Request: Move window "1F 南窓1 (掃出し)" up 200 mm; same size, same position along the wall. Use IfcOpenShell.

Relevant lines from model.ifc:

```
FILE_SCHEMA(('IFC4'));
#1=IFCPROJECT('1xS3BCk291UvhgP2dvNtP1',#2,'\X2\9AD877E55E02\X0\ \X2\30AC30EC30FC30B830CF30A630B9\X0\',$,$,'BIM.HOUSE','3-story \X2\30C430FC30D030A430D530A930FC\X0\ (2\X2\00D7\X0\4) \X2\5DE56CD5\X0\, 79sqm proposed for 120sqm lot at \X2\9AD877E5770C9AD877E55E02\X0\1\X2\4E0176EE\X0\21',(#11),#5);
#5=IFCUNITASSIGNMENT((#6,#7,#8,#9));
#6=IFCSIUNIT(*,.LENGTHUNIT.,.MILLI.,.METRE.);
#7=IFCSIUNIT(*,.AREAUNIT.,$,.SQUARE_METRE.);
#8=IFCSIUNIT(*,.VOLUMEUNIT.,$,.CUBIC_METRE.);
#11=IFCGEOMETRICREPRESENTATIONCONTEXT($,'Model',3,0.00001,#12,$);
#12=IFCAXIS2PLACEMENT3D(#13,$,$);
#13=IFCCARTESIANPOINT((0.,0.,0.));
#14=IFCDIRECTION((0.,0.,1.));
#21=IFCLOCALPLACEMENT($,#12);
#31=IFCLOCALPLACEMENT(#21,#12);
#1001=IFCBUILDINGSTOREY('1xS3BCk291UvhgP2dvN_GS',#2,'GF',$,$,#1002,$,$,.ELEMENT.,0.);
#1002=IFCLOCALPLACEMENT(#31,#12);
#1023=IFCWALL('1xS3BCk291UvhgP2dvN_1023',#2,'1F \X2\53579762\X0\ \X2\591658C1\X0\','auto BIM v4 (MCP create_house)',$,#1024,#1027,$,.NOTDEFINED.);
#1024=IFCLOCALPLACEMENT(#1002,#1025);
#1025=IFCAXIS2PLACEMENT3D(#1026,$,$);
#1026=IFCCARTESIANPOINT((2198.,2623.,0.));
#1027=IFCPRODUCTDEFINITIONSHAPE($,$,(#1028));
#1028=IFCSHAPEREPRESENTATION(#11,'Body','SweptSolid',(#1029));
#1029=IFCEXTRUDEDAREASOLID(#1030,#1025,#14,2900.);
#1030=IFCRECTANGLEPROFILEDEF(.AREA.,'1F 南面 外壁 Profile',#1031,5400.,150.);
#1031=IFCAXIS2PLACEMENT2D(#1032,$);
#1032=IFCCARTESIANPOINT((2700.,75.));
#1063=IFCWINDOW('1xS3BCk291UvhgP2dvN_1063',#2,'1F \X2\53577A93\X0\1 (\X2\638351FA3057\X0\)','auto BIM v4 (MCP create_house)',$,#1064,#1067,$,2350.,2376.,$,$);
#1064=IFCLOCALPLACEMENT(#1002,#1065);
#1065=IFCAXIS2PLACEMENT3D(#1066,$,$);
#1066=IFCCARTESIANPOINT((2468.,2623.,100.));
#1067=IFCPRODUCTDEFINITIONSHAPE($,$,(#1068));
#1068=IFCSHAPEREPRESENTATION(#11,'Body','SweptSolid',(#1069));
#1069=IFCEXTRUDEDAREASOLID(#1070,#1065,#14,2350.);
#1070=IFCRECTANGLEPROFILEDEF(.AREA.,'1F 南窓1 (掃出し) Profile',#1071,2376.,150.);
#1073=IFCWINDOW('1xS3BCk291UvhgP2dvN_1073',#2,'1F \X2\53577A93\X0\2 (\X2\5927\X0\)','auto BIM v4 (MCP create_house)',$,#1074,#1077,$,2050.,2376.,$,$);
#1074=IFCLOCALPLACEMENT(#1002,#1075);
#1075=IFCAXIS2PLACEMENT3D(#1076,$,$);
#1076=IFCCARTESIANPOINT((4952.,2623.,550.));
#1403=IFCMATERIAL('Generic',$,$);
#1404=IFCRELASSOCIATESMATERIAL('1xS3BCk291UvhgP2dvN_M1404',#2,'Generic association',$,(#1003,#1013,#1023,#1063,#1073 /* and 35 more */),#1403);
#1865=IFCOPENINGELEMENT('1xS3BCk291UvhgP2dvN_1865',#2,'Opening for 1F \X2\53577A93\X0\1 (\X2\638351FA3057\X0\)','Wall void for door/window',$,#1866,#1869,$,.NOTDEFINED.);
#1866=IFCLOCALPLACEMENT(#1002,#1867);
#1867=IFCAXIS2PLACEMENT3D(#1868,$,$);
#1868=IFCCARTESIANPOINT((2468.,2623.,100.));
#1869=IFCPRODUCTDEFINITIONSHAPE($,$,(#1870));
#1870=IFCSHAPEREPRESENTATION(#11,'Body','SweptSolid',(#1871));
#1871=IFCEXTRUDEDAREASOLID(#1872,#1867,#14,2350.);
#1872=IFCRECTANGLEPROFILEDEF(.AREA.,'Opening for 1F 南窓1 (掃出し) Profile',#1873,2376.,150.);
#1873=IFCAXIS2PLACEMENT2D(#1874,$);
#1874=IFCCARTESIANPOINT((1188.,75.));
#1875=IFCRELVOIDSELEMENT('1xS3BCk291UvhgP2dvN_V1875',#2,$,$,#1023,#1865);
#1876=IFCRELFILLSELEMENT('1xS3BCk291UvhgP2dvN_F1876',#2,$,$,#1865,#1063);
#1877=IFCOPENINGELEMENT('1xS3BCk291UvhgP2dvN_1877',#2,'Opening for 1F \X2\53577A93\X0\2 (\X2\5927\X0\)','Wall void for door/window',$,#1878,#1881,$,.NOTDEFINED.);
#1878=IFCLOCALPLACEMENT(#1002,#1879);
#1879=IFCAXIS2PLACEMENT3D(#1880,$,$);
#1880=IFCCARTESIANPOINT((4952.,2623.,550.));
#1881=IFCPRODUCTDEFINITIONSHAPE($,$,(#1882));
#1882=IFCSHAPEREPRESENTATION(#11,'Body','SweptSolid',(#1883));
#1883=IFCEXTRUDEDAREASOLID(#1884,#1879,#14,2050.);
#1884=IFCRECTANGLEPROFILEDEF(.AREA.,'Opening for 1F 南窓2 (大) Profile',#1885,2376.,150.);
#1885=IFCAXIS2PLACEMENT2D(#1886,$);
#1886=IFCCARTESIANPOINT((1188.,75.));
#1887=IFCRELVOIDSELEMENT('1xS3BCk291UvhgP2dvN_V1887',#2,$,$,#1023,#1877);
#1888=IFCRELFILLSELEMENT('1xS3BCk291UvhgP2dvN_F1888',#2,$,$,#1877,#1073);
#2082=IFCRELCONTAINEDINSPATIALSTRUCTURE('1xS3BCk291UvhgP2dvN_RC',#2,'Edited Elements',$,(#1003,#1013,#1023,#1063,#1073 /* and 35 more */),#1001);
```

```python
import numpy as np
import ifcopenshell
import ifcopenshell.api.geometry
import ifcopenshell.util.placement
import ifcopenshell.util.unit

model = ifcopenshell.open("model.ifc")
unit_scale = ifcopenshell.util.unit.calculate_unit_scale(model)

window = model.by_guid("1xS3BCk291UvhgP2dvN_1063")
opening = window.FillsVoids[0].RelatingOpeningElement
dz = 0.2 / unit_scale

shift = np.array([0.0, 0.0, dz])
# The window is not placed relative to its opening, so move both.
for product in (opening, window):
    matrix = ifcopenshell.util.placement.get_local_placement(product.ObjectPlacement)
    matrix[:3, 3] += shift
    ifcopenshell.api.geometry.edit_object_placement(model, product=product, matrix=matrix, is_si=False)

print(f"moved by {dz * unit_scale:+.3f} m")

model.write("model_edited.ifc")
```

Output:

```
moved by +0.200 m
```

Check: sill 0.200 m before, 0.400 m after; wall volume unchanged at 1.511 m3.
